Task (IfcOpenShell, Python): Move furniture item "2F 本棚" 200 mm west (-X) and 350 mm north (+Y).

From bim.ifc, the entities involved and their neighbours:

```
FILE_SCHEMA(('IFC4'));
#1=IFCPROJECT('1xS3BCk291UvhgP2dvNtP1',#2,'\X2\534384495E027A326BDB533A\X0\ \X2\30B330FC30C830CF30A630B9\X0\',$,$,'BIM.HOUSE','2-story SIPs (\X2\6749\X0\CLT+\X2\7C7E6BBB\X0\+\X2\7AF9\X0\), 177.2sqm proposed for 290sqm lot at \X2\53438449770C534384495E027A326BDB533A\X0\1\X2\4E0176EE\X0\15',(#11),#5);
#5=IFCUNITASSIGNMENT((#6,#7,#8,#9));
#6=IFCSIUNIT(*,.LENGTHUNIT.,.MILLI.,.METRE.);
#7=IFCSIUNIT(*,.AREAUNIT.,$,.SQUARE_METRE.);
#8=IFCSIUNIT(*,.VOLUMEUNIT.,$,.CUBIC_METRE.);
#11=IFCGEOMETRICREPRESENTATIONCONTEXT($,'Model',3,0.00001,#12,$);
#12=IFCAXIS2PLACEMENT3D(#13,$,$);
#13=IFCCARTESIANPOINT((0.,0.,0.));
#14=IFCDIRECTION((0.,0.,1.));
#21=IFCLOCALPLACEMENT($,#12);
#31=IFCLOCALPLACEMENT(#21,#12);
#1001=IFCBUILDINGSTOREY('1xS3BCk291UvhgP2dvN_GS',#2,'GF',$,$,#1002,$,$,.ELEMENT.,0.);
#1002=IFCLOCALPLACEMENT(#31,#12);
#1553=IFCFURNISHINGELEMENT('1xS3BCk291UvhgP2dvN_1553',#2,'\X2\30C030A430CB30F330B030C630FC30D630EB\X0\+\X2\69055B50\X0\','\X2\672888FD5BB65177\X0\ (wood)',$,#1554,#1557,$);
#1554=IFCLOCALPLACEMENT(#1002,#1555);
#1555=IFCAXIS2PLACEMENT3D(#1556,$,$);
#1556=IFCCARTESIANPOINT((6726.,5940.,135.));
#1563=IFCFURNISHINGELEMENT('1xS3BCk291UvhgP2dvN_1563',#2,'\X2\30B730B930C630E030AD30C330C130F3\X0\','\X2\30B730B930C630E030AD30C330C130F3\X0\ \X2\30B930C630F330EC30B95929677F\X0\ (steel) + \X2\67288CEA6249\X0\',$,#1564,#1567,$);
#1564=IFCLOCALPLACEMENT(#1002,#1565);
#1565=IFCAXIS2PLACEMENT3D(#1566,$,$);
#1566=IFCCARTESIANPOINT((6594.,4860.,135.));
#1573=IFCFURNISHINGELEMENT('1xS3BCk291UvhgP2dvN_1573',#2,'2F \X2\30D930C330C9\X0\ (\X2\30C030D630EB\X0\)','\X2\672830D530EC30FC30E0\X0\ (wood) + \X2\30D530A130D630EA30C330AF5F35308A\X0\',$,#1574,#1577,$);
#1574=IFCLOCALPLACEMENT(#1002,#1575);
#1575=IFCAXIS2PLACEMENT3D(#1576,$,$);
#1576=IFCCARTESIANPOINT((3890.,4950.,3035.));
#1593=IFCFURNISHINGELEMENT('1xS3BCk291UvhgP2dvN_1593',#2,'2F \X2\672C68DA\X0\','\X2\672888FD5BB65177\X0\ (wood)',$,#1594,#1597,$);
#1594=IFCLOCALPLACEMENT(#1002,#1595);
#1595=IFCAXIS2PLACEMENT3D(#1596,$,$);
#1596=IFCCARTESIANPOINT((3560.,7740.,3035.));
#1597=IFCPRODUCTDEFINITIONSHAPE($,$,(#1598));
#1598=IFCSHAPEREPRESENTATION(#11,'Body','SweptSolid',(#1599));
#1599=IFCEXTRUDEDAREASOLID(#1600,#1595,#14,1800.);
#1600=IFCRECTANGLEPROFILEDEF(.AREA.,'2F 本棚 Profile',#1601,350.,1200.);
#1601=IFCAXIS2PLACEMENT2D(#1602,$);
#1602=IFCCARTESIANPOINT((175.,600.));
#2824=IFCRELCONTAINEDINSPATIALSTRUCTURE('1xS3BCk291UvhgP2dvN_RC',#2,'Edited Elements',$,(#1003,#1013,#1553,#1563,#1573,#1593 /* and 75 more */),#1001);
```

```python
import ifcopenshell
import ifcopenshell.api.geometry
import ifcopenshell.util.placement
import ifcopenshell.util.unit

model = ifcopenshell.open("bim.ifc")
unit_scale = ifcopenshell.util.unit.calculate_unit_scale(model)

item = model.by_guid("1xS3BCk291UvhgP2dvN_1593")
matrix = ifcopenshell.util.placement.get_local_placement(item.ObjectPlacement)
matrix[0, 3] -= 0.2 / unit_scale
matrix[1, 3] += 0.35 / unit_scale
ifcopenshell.api.geometry.edit_object_placement(model, product=item, matrix=matrix, is_si=False)

print(ifcopenshell.util.placement.get_local_placement(item.ObjectPlacement).round(3) + 0.0)

model.write("bim_v2.ifc")
```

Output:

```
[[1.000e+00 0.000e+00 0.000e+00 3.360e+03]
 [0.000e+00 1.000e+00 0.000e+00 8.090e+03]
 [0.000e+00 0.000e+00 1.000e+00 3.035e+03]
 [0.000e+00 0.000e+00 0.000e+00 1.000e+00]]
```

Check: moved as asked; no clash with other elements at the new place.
